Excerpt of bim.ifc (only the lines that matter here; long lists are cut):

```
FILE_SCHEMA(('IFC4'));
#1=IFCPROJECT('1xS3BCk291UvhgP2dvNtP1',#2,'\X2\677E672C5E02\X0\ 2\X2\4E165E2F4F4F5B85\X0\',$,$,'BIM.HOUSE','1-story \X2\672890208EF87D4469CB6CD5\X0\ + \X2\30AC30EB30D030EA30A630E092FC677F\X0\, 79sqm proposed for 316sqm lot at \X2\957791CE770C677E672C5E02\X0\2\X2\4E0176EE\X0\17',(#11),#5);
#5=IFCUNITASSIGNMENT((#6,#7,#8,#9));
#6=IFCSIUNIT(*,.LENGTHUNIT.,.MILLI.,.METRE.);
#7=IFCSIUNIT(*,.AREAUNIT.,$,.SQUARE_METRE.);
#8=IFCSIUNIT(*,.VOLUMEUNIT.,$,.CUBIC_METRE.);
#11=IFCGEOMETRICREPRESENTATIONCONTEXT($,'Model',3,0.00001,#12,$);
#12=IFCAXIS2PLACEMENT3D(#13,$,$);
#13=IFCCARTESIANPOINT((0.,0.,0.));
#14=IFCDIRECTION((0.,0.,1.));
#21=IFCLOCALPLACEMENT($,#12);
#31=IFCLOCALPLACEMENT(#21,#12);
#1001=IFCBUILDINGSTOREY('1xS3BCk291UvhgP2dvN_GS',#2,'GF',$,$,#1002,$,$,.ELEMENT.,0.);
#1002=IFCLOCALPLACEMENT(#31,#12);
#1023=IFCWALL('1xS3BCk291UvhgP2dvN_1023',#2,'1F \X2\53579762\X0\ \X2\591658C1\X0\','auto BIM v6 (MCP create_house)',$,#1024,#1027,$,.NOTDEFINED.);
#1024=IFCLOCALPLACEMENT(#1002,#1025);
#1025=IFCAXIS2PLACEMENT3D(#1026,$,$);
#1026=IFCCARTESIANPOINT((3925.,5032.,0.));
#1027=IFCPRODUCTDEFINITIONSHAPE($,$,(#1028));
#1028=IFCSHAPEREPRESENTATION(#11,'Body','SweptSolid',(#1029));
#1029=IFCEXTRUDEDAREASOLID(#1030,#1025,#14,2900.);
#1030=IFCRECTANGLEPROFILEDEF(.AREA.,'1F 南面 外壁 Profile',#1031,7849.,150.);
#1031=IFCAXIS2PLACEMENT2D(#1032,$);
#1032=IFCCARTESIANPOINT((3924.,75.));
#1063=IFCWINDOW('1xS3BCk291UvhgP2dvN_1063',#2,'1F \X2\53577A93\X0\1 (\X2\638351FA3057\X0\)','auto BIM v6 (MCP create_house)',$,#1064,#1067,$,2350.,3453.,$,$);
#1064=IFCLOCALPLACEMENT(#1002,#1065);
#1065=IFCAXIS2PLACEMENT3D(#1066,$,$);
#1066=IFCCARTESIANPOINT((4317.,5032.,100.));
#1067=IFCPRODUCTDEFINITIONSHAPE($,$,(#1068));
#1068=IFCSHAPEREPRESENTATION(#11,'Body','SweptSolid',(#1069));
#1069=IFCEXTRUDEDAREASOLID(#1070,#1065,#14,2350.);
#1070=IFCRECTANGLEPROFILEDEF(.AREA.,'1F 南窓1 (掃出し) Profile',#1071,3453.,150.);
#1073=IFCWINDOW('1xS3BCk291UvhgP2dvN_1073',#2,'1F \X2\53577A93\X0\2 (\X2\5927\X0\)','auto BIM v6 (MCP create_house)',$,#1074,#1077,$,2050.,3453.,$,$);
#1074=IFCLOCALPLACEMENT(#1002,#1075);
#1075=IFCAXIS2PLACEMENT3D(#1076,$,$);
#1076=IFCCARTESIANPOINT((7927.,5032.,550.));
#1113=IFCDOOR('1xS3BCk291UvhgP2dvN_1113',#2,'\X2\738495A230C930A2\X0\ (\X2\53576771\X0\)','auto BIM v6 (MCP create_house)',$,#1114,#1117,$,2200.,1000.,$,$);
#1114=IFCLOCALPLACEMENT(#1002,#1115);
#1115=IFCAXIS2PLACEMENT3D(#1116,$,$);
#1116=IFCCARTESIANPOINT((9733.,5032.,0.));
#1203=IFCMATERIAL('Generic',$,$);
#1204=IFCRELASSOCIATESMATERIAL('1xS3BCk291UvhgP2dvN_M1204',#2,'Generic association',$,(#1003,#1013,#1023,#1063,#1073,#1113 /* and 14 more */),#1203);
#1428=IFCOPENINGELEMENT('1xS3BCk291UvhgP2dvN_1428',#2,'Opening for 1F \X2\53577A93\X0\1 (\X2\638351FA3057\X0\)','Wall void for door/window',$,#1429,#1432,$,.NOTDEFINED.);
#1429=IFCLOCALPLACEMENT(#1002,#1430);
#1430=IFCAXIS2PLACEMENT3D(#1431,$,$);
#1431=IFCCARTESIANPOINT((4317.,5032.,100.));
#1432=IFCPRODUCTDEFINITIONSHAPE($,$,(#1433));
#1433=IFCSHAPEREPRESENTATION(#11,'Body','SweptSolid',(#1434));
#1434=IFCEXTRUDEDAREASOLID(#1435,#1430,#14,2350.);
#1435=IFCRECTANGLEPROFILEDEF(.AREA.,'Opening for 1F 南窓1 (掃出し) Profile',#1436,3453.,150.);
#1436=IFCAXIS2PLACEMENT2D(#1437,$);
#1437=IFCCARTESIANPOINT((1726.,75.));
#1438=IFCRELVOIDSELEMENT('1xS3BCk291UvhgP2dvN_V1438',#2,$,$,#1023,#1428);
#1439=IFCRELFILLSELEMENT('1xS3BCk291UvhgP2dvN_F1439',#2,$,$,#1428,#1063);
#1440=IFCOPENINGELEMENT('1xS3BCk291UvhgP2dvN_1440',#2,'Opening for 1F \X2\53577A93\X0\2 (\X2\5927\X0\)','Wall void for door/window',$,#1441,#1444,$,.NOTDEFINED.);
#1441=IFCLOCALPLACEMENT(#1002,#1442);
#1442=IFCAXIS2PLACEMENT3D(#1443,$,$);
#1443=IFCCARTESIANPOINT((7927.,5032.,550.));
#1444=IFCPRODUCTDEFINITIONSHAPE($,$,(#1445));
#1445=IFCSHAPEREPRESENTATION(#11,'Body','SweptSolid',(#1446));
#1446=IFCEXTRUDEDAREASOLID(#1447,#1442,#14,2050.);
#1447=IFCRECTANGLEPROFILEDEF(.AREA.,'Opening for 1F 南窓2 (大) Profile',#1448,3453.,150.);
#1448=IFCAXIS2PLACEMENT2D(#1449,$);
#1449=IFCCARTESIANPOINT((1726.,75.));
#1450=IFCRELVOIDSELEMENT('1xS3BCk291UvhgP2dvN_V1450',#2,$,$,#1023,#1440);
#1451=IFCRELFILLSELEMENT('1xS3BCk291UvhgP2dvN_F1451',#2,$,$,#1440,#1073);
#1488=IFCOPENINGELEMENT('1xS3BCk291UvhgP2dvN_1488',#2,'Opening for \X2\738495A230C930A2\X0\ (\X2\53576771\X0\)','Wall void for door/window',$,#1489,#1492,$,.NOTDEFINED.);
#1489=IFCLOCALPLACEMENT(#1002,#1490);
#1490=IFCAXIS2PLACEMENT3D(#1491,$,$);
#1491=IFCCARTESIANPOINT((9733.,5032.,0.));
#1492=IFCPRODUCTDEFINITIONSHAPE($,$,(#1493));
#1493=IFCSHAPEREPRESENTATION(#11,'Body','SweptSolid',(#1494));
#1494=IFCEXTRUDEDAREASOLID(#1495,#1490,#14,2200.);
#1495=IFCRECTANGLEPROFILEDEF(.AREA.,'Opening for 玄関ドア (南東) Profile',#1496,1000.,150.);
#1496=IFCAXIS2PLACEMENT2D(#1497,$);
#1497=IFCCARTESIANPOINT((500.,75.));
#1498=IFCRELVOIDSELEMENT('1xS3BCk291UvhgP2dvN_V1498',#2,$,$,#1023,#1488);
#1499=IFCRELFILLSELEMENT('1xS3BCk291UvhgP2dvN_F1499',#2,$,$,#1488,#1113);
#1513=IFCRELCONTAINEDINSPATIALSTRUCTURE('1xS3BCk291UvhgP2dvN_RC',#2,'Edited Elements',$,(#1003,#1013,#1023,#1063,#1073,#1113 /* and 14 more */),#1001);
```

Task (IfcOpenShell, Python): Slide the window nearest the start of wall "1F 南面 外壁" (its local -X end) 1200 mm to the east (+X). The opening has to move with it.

```python
import ifcopenshell
import ifcopenshell.api.geometry
import ifcopenshell.util.placement
import ifcopenshell.util.unit

model = ifcopenshell.open("bim.ifc")
unit_scale = ifcopenshell.util.unit.calculate_unit_scale(model)

window = model.by_guid("1xS3BCk291UvhgP2dvN_1063")
opening = window.FillsVoids[0].RelatingOpeningElement
wall = opening.VoidsElements[0].RelatingBuildingElement

wall_matrix = ifcopenshell.util.placement.get_local_placement(wall.ObjectPlacement)
shift = wall_matrix[:3, 0] * 1.2 / unit_scale
before = ifcopenshell.util.placement.get_local_placement(window.ObjectPlacement)[:3, 3].copy()

# The window is not placed relative to its opening, so move both.
for product in (opening, window):
    matrix = ifcopenshell.util.placement.get_local_placement(product.ObjectPlacement)
    matrix[:3, 3] += shift
    ifcopenshell.api.geometry.edit_object_placement(model, product=product, matrix=matrix, is_si=False)

after = ifcopenshell.util.placement.get_local_placement(window.ObjectPlacement)[:3, 3]
print("window moved by", (after - before).round(3) + 0.0)

model.write("bim-out.ifc")
```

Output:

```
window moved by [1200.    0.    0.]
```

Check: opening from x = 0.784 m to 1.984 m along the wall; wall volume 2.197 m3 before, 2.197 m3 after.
